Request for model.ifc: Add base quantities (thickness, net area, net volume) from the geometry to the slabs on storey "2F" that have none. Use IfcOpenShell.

First a look at what the model holds.

```python
import ifcopenshell
import ifcopenshell.util.element
import ifcopenshell.util.unit

model = ifcopenshell.open("model.ifc")
print(model.schema)
for unit_type in ("LENGTHUNIT", "AREAUNIT", "VOLUMEUNIT"):
    print(unit_type, ifcopenshell.util.unit.calculate_unit_scale(model, unit_type))
storey = next(s for s in model.by_type("IfcBuildingStorey") if s.Name == "2F")
slabs = [e for e in ifcopenshell.util.element.get_decomposition(storey) if e.is_a("IfcSlab")]
for e in sorted(slabs, key=lambda e: e.id()):
    print(e.id(), e.is_a(), e.Name, list(ifcopenshell.util.element.get_psets(e, qtos_only=True)), sep=" | ")
```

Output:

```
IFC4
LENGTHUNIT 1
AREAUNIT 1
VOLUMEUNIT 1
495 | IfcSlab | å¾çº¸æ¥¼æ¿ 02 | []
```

```python
import ifcopenshell
import ifcopenshell.api.pset
import ifcopenshell.geom
import ifcopenshell.util.element
import ifcopenshell.util.shape
import ifcopenshell.util.unit

model = ifcopenshell.open("model.ifc")
unit_scale = ifcopenshell.util.unit.calculate_unit_scale(model)
area_scale = ifcopenshell.util.unit.calculate_unit_scale(model, "AREAUNIT")
volume_scale = ifcopenshell.util.unit.calculate_unit_scale(model, "VOLUMEUNIT")
settings = ifcopenshell.geom.settings()

storey = next(s for s in model.by_type("IfcBuildingStorey") if s.Name == "2F")
slabs = [e for e in ifcopenshell.util.element.get_decomposition(storey) if e.is_a("IfcSlab")]

for e in sorted(slabs, key=lambda e: e.id()):
    if ifcopenshell.util.element.get_psets(e, qtos_only=True, should_inherit=False):
        continue
    # Geometry comes back in metres, in the element's own axes.
    shape = ifcopenshell.geom.create_shape(settings, e)
    values = {
        "Width": ifcopenshell.util.shape.get_z(shape.geometry) / unit_scale,
        "NetArea": ifcopenshell.util.shape.get_footprint_area(shape.geometry) / area_scale,
        "NetVolume": ifcopenshell.util.shape.get_volume(shape.geometry) / volume_scale,
    }
    qto = ifcopenshell.api.pset.add_qto(model, product=e, name="Qto_SlabBaseQuantities")
    ifcopenshell.api.pset.edit_qto(model, qto=qto, properties=values)
    print(e.id(), {k: round(v, 3) for k, v in values.items()})

model.write("model_updated.ifc")
```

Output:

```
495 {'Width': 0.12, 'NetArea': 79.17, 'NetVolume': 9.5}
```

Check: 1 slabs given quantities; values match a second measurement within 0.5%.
